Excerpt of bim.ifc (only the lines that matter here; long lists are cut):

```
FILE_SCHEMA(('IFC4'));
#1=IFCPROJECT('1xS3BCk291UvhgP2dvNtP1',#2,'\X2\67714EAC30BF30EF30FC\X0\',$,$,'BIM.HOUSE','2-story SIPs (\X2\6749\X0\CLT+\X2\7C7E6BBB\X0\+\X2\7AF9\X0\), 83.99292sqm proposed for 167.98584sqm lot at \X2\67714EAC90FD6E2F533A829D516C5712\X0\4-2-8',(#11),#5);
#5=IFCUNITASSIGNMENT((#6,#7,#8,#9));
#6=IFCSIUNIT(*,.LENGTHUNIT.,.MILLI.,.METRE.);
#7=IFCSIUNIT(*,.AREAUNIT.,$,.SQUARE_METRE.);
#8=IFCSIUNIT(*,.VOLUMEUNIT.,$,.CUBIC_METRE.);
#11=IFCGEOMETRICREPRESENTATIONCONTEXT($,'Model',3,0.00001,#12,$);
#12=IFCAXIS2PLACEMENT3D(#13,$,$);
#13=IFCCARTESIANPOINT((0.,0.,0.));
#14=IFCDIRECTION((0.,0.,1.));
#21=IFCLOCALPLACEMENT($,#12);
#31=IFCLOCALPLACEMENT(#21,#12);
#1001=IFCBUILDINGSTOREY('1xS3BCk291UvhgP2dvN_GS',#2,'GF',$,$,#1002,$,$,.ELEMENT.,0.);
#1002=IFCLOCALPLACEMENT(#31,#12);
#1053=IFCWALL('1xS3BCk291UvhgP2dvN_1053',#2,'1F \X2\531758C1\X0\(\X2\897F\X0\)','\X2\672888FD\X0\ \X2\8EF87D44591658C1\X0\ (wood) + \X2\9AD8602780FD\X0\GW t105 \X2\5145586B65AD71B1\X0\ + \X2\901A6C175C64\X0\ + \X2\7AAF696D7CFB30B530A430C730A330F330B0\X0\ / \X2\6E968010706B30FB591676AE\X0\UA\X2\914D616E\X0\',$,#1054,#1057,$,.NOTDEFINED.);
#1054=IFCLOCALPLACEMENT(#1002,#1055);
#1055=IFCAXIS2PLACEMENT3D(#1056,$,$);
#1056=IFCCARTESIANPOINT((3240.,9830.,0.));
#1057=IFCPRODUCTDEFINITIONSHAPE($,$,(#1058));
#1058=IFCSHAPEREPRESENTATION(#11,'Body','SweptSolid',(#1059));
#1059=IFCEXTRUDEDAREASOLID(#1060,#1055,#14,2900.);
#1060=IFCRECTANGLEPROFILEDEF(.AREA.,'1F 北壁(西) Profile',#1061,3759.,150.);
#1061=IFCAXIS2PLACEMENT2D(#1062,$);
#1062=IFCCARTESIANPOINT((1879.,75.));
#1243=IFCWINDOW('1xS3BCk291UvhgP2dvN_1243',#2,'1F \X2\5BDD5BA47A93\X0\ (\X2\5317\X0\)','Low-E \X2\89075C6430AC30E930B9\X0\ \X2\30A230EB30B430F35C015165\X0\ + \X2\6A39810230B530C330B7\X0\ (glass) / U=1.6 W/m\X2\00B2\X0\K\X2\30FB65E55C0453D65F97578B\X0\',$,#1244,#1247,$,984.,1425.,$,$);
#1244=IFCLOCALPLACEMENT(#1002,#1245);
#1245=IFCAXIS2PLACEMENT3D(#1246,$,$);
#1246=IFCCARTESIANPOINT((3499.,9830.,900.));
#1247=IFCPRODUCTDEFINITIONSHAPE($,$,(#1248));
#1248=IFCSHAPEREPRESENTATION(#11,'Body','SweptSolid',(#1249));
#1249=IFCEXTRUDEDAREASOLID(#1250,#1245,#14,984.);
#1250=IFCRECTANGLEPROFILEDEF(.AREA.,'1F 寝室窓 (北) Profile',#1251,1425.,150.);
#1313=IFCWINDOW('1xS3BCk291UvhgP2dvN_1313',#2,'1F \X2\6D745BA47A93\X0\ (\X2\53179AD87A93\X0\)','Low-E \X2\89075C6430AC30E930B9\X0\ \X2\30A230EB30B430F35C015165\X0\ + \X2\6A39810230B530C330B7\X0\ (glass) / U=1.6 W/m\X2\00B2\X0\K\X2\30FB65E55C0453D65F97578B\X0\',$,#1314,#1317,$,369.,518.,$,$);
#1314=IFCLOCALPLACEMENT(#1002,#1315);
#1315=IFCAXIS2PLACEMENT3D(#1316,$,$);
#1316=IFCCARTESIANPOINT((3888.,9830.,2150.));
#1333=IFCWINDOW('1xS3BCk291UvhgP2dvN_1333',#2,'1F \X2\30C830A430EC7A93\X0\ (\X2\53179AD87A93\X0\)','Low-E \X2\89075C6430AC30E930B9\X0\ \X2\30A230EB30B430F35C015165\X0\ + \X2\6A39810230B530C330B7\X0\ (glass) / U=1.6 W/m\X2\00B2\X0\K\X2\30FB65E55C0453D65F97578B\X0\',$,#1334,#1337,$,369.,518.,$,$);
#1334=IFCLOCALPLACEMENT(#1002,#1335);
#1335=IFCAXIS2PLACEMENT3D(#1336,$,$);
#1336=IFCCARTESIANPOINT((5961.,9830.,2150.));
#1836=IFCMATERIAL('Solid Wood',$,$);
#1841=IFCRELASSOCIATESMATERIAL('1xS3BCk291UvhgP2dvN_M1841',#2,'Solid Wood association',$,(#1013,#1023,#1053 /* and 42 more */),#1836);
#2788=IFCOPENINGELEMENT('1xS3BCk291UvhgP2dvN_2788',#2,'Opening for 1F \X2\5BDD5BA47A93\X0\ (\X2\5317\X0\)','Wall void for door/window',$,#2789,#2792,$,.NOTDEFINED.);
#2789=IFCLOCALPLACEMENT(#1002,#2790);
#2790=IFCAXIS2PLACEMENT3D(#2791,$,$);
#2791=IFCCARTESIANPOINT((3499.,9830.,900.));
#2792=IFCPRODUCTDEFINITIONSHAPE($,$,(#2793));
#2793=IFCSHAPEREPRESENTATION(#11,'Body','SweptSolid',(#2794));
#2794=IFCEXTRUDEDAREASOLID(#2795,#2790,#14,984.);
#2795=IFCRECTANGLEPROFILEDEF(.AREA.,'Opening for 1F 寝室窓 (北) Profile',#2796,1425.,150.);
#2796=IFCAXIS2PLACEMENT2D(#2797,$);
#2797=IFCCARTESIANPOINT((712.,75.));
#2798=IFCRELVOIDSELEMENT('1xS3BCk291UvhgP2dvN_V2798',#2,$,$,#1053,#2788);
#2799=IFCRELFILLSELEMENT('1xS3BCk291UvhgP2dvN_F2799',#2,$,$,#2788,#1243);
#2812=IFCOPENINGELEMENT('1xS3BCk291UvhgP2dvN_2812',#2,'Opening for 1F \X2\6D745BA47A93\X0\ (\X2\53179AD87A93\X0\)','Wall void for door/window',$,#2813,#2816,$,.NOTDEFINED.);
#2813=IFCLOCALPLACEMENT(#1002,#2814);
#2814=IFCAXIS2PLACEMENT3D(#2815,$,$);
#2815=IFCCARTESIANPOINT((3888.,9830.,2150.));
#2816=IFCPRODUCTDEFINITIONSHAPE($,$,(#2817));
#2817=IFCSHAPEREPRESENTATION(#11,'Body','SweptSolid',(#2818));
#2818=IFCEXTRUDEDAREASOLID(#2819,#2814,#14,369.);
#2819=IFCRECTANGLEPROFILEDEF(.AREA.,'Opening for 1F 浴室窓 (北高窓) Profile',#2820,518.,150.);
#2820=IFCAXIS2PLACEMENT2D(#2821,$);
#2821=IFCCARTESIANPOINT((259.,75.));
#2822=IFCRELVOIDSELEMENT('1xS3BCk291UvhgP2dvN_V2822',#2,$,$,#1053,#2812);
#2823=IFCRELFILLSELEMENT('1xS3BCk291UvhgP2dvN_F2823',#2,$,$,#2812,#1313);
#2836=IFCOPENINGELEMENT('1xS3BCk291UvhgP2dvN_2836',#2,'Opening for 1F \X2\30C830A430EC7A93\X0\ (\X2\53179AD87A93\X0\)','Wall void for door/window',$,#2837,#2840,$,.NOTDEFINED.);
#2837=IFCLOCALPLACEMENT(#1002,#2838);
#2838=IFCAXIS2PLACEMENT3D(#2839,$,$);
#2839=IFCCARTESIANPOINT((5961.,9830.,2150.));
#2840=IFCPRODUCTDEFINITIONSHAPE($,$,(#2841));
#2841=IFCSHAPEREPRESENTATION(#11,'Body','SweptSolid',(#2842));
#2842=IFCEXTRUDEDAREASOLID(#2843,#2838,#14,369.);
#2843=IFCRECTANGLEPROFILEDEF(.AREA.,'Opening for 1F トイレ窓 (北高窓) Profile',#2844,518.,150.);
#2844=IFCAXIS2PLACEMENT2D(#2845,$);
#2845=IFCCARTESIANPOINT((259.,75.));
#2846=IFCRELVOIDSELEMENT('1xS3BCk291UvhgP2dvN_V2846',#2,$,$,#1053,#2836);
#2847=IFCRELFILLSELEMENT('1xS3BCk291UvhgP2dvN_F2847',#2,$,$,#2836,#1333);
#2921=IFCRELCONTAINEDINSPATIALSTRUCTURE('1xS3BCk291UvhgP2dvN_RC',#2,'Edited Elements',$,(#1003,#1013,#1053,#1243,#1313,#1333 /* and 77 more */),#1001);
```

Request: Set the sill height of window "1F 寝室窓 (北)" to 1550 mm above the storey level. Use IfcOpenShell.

```python
import numpy as np
import ifcopenshell
import ifcopenshell.api.geometry
import ifcopenshell.geom
import ifcopenshell.util.element
import ifcopenshell.util.placement
import ifcopenshell.util.shape
import ifcopenshell.util.unit

model = ifcopenshell.open("bim.ifc")
unit_scale = ifcopenshell.util.unit.calculate_unit_scale(model)

window = model.by_guid("1xS3BCk291UvhgP2dvN_1243")
opening = window.FillsVoids[0].RelatingOpeningElement
storey = ifcopenshell.util.element.get_container(window, ifc_class="IfcBuildingStorey")
level = ifcopenshell.util.placement.get_local_placement(storey.ObjectPlacement)[2, 3]

# The opening's origin need not be at the sill, so measure its lowest point.
shape = ifcopenshell.geom.create_shape(ifcopenshell.geom.settings(), opening)
bottom = ifcopenshell.util.shape.get_shape_bottom_elevation(shape, shape.geometry) / unit_scale
dz = level + 1550.0 - bottom

shift = np.array([0.0, 0.0, dz])
# The window is not placed relative to its opening, so move both.
for product in (opening, window):
    matrix = ifcopenshell.util.placement.get_local_placement(product.ObjectPlacement)
    matrix[:3, 3] += shift
    ifcopenshell.api.geometry.edit_object_placement(model, product=product, matrix=matrix, is_si=False)

print(f"moved by {dz * unit_scale:+.3f} m")

model.write("bim_edited.ifc")
```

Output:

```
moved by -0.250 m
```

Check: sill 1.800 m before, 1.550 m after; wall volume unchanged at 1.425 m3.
